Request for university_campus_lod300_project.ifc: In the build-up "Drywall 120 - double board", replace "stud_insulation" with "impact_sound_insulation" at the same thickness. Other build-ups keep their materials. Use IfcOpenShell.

First a look at what the model holds.

```python
import ifcopenshell
import ifcopenshell.util.element

model = ifcopenshell.open("university_campus_lod300_project.ifc")
print(model.schema)
for layer_set in model.by_type("IfcMaterialLayerSet"):
    if layer_set.LayerSetName == "Drywall 120 - double board":
        for layer in layer_set.MaterialLayers:
            print(layer.id(), layer.Material and layer.Material.Name, layer.LayerThickness, sep=" | ")
        print(len(ifcopenshell.util.element.get_elements_by_material(model, layer_set)), "elements and types use it")
print(sorted(m.Name for m in model.by_type("IfcMaterial") if m.Name)[:60])
```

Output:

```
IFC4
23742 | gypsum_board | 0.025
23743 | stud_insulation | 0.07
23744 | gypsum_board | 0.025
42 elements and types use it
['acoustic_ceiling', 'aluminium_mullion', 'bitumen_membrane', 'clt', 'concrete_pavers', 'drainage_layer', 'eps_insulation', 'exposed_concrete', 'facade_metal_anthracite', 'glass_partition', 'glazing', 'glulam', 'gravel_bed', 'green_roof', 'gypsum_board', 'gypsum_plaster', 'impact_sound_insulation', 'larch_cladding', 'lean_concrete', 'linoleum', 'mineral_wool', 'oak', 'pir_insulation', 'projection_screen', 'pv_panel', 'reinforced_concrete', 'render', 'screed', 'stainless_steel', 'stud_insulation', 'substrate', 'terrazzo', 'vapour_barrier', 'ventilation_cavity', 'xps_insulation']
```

```python
import ifcopenshell
import ifcopenshell.api.material

model = ifcopenshell.open("university_campus_lod300_project.ifc")

layer_set = next(s for s in model.by_type("IfcMaterialLayerSet") if s.LayerSetName == "Drywall 120 - double board")
layer = next(l for l in layer_set.MaterialLayers if l.Material and l.Material.Name == "stud_insulation")
material = next(m for m in model.by_type("IfcMaterial") if m.Name == "impact_sound_insulation")

# Point this one layer at the other material; renaming the old one would change it everywhere.
ifcopenshell.api.material.edit_layer(model, layer=layer, attributes={"Name": material.Name}, material=material)

print([l.Material.Name if l.Material else None for l in layer_set.MaterialLayers])

model.write("university_campus_lod300_project_updated.ifc")
```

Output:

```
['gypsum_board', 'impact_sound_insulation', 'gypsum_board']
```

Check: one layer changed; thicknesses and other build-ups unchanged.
